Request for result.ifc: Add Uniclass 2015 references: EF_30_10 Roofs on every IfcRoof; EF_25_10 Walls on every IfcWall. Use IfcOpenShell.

First a look at what the model holds.

```python
import ifcopenshell

model = ifcopenshell.open("result.ifc")
print(model.schema)
print("classifications:", [c.Name for c in model.by_type("IfcClassification")])
for ifc_class in ("IfcDoor", "IfcRoof", "IfcStair", "IfcWall", "IfcWindow"):
    print(ifc_class, len(model.by_type(ifc_class)))
```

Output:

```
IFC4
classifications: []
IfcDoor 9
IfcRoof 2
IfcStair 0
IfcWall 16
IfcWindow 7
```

```python
import ifcopenshell
import ifcopenshell.api.classification

model = ifcopenshell.open("result.ifc")

system = ifcopenshell.api.classification.add_classification(model, classification="Uniclass 2015")

codes = {
    "IfcRoof": ("EF_30_10", "Roofs"),
    "IfcWall": ("EF_25_10", "Walls"),
}
for ifc_class, (code, name) in codes.items():
    products = model.by_type(ifc_class)
    ifcopenshell.api.classification.add_reference(
        model, products=products, classification=system, identification=code, name=name
    )
    print(code, len(products))

model.write("result-out.ifc")
```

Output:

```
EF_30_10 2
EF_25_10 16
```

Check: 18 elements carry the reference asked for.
